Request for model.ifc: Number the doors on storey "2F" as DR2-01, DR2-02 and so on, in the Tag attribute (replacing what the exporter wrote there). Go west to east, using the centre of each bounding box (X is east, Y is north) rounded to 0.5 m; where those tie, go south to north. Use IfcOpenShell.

First a look at what the model holds.

```python
import ifcopenshell
import ifcopenshell.util.element
import ifcopenshell.util.placement

model = ifcopenshell.open("model.ifc")
print(model.schema)
storey = next(s for s in model.by_type("IfcBuildingStorey") if s.Name == "2F")
doors = [e for e in ifcopenshell.util.element.get_decomposition(storey) if e.is_a("IfcDoor")]
for e in sorted(doors, key=lambda e: e.id()):
    origin = ifcopenshell.util.placement.get_local_placement(e.ObjectPlacement)[:3, 3]
    print(e.id(), e.Tag, e.Name, origin.round(2) + 0.0, sep=" | ")
```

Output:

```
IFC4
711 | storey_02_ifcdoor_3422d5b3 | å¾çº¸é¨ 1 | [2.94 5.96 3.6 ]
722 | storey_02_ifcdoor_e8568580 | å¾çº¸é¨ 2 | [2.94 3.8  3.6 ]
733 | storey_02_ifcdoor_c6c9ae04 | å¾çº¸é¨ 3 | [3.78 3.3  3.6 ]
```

```python
import ifcopenshell
import ifcopenshell.geom
import ifcopenshell.util.element
import ifcopenshell.util.shape

model = ifcopenshell.open("model.ifc")
settings = ifcopenshell.geom.settings()
settings.set("use-world-coords", True)


def centre(element):
    shape = ifcopenshell.geom.create_shape(settings, element)
    return ifcopenshell.util.shape.get_bbox_centroid(shape.geometry)


storey = next(s for s in model.by_type("IfcBuildingStorey") if s.Name == "2F")
doors = [e for e in ifcopenshell.util.element.get_decomposition(storey) if e.is_a("IfcDoor")]

# Insertion points can sit at a corner or the storey origin, so sort by the geometry (in metres).
centres = {e: centre(e) for e in doors}
doors.sort(key=lambda e: (round(centres[e][0] / 0.5), centres[e][1]))

for i, e in enumerate(doors, start=1):
    number = f"DR2-{i:02d}"
    e.Tag = number
    print(e.id(), number)

model.write("model_updated.ifc")
```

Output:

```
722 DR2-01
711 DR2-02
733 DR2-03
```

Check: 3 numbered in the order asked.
